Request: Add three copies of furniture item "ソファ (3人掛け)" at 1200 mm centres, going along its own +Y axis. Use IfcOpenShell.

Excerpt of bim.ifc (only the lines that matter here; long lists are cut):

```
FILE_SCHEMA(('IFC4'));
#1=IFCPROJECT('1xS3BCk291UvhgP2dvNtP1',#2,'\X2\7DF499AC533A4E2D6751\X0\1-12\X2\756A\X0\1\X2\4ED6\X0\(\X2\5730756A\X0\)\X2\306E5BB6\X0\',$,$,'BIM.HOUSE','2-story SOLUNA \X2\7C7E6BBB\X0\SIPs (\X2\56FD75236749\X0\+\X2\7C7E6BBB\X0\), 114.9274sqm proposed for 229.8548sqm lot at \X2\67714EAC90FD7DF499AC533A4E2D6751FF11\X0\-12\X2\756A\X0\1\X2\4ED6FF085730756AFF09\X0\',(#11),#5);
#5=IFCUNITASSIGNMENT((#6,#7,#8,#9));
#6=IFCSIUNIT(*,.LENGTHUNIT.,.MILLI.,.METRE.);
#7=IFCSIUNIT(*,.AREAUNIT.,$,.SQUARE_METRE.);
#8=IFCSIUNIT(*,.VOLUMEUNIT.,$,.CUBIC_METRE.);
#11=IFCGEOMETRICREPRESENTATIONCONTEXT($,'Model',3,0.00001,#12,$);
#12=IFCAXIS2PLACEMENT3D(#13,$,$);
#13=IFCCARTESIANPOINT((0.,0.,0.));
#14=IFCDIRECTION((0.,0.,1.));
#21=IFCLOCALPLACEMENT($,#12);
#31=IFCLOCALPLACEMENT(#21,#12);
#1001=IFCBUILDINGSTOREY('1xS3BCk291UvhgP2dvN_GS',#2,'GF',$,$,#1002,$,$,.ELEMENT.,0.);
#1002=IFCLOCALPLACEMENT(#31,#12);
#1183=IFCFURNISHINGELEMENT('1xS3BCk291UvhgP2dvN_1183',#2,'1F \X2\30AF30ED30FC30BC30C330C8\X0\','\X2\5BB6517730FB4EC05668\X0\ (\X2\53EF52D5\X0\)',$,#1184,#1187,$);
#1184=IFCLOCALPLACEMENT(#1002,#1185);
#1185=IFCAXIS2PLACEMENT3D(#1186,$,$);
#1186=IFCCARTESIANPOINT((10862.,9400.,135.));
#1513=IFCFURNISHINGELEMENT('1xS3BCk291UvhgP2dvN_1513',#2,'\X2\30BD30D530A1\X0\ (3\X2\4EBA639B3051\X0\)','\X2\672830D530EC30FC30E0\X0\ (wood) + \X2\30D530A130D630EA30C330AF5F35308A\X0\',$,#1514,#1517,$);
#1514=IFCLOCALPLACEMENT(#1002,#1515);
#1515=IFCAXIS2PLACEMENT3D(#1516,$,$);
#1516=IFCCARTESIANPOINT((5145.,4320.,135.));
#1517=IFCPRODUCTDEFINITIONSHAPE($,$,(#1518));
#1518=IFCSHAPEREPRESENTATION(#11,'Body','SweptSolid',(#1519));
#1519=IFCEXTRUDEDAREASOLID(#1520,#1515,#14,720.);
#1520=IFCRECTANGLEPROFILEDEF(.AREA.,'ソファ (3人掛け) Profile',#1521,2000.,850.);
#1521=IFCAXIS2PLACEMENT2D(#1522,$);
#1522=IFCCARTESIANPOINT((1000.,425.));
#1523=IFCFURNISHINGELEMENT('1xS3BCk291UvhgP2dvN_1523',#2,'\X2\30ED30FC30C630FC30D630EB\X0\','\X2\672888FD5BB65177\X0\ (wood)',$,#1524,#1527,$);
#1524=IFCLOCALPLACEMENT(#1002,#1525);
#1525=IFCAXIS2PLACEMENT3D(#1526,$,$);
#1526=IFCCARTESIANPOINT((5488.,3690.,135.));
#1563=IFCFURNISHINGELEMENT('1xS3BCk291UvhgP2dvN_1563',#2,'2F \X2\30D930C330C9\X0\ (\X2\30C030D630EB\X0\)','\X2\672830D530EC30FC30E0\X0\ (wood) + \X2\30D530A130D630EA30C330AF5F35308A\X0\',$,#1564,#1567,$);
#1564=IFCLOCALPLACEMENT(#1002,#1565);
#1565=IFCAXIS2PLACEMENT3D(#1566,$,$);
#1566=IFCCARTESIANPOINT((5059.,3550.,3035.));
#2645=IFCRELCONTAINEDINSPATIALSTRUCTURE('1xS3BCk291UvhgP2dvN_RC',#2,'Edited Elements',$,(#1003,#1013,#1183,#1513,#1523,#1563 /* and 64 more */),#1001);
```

```python
import ifcopenshell
import ifcopenshell.api.geometry
import ifcopenshell.api.root
import ifcopenshell.util.element
import ifcopenshell.util.placement
import ifcopenshell.util.unit

model = ifcopenshell.open("bim.ifc")
unit_scale = ifcopenshell.util.unit.calculate_unit_scale(model)


def reuse_history(source, copy):
    """copy_class also copies each property set's owner history, people and application; keep the originals."""
    for rel in copy.IsDefinedBy:
        if rel.is_a("IfcRelDefinesByProperties") and (history := rel.RelatingPropertyDefinition.OwnerHistory):
            rel.RelatingPropertyDefinition.OwnerHistory = source.OwnerHistory
            ifcopenshell.util.element.remove_deep2(model, history)


source = model.by_id(1513)
base = ifcopenshell.util.placement.get_local_placement(source.ObjectPlacement)
step = base[:3, 1] * 1.2 / unit_scale

for i in range(1, 4):
    copy = ifcopenshell.api.root.copy_class(model, product=source)
    copy.Representation = ifcopenshell.util.element.copy_deep(
        model, source.Representation, exclude=["IfcGeometricRepresentationContext", "IfcRepresentationMap"]
    )
    reuse_history(source, copy)
    matrix = base.copy()
    matrix[:3, 3] += i * step
    print("added at", matrix[:3, 3].round(3) + 0.0)
    ifcopenshell.api.geometry.edit_object_placement(model, product=copy, matrix=matrix, is_si=False)

model.write("bim_updated.ifc")
```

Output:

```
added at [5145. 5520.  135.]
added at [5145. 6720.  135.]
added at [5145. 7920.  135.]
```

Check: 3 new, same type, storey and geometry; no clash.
